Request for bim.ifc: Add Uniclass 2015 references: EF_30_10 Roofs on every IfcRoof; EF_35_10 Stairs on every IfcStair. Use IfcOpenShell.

First a look at what the model holds.

```python
import ifcopenshell

model = ifcopenshell.open("bim.ifc")
print(model.schema)
print("classifications:", [c.Name for c in model.by_type("IfcClassification")])
for ifc_class in ("IfcDoor", "IfcRoof", "IfcStair", "IfcWall", "IfcWindow"):
    print(ifc_class, len(model.by_type(ifc_class)))
```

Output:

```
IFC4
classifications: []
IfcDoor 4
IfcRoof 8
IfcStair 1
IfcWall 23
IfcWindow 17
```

```python
import ifcopenshell
import ifcopenshell.api.classification

model = ifcopenshell.open("bim.ifc")

system = ifcopenshell.api.classification.add_classification(model, classification="Uniclass 2015")

codes = {
    "IfcRoof": ("EF_30_10", "Roofs"),
    "IfcStair": ("EF_35_10", "Stairs"),
}
for ifc_class, (code, name) in codes.items():
    products = model.by_type(ifc_class)
    ifcopenshell.api.classification.add_reference(
        model, products=products, classification=system, identification=code, name=name
    )
    print(code, len(products))

model.write("bim_edited.ifc")
```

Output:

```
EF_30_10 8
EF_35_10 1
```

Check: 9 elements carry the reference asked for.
